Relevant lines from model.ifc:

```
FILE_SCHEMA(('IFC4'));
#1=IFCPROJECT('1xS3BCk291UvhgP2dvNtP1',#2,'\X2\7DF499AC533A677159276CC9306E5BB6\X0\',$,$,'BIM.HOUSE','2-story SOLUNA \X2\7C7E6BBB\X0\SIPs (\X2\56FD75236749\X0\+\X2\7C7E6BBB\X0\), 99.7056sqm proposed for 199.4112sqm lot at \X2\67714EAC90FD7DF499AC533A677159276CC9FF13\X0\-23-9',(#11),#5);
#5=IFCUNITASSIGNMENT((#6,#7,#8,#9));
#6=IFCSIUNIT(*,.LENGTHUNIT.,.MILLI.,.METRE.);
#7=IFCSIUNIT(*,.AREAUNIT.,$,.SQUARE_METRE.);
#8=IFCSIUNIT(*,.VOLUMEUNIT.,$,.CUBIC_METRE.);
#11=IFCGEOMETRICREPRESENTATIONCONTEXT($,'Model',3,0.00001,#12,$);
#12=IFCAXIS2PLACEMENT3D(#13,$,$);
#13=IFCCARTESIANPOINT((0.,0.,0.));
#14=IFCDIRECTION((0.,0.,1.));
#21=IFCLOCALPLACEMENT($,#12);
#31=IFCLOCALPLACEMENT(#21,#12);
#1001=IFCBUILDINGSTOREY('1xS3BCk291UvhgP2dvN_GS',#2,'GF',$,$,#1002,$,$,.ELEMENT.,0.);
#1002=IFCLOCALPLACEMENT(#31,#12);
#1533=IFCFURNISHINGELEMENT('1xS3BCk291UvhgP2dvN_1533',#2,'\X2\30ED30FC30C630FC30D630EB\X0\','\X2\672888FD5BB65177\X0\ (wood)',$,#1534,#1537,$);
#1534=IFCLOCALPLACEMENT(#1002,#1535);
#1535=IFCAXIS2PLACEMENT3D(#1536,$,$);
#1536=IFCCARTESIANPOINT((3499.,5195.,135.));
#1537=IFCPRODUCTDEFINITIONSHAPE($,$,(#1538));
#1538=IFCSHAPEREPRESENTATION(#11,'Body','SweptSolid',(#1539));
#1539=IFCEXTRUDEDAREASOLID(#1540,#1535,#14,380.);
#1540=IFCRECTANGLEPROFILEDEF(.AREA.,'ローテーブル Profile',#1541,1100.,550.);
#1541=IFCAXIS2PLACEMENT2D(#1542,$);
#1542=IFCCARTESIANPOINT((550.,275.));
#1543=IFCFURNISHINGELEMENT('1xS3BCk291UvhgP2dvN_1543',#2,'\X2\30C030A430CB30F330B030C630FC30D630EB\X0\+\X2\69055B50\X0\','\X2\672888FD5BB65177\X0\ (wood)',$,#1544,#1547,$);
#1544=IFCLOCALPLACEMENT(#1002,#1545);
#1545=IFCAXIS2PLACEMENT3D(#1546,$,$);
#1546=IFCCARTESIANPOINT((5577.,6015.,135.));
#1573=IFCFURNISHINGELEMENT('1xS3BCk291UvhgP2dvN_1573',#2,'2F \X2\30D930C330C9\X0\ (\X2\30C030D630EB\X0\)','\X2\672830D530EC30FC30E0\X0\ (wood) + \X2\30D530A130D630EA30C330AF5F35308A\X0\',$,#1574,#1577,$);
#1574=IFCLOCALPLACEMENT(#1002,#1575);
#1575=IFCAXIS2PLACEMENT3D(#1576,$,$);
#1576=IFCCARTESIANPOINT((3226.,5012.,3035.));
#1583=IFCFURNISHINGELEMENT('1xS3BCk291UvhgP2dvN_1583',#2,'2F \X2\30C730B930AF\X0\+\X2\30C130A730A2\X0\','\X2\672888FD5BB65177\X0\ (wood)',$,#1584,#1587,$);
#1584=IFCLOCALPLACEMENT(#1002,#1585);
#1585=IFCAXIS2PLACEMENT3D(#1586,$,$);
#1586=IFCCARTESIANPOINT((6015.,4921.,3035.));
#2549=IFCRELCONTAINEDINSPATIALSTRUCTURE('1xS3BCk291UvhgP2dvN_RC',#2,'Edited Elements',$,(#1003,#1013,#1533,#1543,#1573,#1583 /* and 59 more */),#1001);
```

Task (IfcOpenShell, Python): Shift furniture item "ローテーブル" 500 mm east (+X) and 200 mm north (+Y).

```python
import ifcopenshell
import ifcopenshell.api.geometry
import ifcopenshell.util.placement
import ifcopenshell.util.unit

model = ifcopenshell.open("model.ifc")
unit_scale = ifcopenshell.util.unit.calculate_unit_scale(model)

item = model.by_id(1533)
matrix = ifcopenshell.util.placement.get_local_placement(item.ObjectPlacement)
matrix[0, 3] += 0.5 / unit_scale
matrix[1, 3] += 0.2 / unit_scale
ifcopenshell.api.geometry.edit_object_placement(model, product=item, matrix=matrix, is_si=False)

print(ifcopenshell.util.placement.get_local_placement(item.ObjectPlacement).round(3) + 0.0)

model.write("model_rev.ifc")
```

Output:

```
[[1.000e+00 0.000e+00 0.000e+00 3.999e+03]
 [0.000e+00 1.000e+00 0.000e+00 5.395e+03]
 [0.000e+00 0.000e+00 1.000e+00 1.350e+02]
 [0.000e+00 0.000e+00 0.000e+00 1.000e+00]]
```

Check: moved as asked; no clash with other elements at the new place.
